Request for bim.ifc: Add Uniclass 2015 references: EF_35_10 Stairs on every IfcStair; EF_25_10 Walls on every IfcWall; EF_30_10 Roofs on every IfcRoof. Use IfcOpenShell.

First a look at what the model holds.

```python
import ifcopenshell

model = ifcopenshell.open("bim.ifc")
print(model.schema)
print("classifications:", [c.Name for c in model.by_type("IfcClassification")])
for ifc_class in ("IfcDoor", "IfcRoof", "IfcStair", "IfcWall", "IfcWindow"):
    print(ifc_class, len(model.by_type(ifc_class)))
```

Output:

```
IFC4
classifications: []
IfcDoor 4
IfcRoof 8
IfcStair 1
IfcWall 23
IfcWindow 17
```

```python
import ifcopenshell
import ifcopenshell.api.classification

model = ifcopenshell.open("bim.ifc")

system = ifcopenshell.api.classification.add_classification(model, classification="Uniclass 2015")

codes = {
    "IfcStair": ("EF_35_10", "Stairs"),
    "IfcWall": ("EF_25_10", "Walls"),
    "IfcRoof": ("EF_30_10", "Roofs"),
}
for ifc_class, (code, name) in codes.items():
    products = model.by_type(ifc_class)
    ifcopenshell.api.classification.add_reference(
        model, products=products, classification=system, identification=code, name=name
    )
    print(code, len(products))

model.write("bim_rev.ifc")
```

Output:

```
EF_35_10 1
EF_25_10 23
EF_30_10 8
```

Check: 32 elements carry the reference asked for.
